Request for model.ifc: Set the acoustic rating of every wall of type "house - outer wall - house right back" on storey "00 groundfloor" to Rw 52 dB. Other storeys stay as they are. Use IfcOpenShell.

First a look at what the model holds.

```python
import ifcopenshell
import ifcopenshell.util.element

model = ifcopenshell.open("model.ifc")
print(model.schema)
storey = next(s for s in model.by_type("IfcBuildingStorey") if s.Name == "00 groundfloor")
walls = [e for e in ifcopenshell.util.element.get_decomposition(storey) if e.is_a("IfcWall")]
seen = {}
for e in walls:
    element_type = ifcopenshell.util.element.get_type(e)
    key = (element_type.Name if element_type != e and element_type else None, ifcopenshell.util.element.get_pset(e, "Pset_WallCommon", "AcousticRating"))
    seen[key] = seen.get(key, 0) + 1
for (name, value), count in sorted(seen.items(), key=str):
    print(count, "x", name, "|", value)
```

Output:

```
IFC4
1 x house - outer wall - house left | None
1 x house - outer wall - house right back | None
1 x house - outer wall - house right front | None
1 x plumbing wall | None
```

```python
import ifcopenshell
import ifcopenshell.api.pset
import ifcopenshell.util.element

model = ifcopenshell.open("model.ifc")

storey = next(s for s in model.by_type("IfcBuildingStorey") if s.Name == "00 groundfloor")
walls = [e for e in ifcopenshell.util.element.get_decomposition(storey) if e.is_a("IfcWall")]

count = 0
for e in walls:
    element_type = ifcopenshell.util.element.get_type(e)
    if element_type in (None, e) or element_type.Name != "house - outer wall - house right back":
        continue
    # add_pset returns the element's existing set when there is one.
    pset = ifcopenshell.api.pset.add_pset(model, product=e, name="Pset_WallCommon")
    ifcopenshell.api.pset.edit_pset(model, pset=pset, properties={"AcousticRating": "Rw 52 dB"})
    count += 1

print(count, "walls updated")

model.write("model-out.ifc")
```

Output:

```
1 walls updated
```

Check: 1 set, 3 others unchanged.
